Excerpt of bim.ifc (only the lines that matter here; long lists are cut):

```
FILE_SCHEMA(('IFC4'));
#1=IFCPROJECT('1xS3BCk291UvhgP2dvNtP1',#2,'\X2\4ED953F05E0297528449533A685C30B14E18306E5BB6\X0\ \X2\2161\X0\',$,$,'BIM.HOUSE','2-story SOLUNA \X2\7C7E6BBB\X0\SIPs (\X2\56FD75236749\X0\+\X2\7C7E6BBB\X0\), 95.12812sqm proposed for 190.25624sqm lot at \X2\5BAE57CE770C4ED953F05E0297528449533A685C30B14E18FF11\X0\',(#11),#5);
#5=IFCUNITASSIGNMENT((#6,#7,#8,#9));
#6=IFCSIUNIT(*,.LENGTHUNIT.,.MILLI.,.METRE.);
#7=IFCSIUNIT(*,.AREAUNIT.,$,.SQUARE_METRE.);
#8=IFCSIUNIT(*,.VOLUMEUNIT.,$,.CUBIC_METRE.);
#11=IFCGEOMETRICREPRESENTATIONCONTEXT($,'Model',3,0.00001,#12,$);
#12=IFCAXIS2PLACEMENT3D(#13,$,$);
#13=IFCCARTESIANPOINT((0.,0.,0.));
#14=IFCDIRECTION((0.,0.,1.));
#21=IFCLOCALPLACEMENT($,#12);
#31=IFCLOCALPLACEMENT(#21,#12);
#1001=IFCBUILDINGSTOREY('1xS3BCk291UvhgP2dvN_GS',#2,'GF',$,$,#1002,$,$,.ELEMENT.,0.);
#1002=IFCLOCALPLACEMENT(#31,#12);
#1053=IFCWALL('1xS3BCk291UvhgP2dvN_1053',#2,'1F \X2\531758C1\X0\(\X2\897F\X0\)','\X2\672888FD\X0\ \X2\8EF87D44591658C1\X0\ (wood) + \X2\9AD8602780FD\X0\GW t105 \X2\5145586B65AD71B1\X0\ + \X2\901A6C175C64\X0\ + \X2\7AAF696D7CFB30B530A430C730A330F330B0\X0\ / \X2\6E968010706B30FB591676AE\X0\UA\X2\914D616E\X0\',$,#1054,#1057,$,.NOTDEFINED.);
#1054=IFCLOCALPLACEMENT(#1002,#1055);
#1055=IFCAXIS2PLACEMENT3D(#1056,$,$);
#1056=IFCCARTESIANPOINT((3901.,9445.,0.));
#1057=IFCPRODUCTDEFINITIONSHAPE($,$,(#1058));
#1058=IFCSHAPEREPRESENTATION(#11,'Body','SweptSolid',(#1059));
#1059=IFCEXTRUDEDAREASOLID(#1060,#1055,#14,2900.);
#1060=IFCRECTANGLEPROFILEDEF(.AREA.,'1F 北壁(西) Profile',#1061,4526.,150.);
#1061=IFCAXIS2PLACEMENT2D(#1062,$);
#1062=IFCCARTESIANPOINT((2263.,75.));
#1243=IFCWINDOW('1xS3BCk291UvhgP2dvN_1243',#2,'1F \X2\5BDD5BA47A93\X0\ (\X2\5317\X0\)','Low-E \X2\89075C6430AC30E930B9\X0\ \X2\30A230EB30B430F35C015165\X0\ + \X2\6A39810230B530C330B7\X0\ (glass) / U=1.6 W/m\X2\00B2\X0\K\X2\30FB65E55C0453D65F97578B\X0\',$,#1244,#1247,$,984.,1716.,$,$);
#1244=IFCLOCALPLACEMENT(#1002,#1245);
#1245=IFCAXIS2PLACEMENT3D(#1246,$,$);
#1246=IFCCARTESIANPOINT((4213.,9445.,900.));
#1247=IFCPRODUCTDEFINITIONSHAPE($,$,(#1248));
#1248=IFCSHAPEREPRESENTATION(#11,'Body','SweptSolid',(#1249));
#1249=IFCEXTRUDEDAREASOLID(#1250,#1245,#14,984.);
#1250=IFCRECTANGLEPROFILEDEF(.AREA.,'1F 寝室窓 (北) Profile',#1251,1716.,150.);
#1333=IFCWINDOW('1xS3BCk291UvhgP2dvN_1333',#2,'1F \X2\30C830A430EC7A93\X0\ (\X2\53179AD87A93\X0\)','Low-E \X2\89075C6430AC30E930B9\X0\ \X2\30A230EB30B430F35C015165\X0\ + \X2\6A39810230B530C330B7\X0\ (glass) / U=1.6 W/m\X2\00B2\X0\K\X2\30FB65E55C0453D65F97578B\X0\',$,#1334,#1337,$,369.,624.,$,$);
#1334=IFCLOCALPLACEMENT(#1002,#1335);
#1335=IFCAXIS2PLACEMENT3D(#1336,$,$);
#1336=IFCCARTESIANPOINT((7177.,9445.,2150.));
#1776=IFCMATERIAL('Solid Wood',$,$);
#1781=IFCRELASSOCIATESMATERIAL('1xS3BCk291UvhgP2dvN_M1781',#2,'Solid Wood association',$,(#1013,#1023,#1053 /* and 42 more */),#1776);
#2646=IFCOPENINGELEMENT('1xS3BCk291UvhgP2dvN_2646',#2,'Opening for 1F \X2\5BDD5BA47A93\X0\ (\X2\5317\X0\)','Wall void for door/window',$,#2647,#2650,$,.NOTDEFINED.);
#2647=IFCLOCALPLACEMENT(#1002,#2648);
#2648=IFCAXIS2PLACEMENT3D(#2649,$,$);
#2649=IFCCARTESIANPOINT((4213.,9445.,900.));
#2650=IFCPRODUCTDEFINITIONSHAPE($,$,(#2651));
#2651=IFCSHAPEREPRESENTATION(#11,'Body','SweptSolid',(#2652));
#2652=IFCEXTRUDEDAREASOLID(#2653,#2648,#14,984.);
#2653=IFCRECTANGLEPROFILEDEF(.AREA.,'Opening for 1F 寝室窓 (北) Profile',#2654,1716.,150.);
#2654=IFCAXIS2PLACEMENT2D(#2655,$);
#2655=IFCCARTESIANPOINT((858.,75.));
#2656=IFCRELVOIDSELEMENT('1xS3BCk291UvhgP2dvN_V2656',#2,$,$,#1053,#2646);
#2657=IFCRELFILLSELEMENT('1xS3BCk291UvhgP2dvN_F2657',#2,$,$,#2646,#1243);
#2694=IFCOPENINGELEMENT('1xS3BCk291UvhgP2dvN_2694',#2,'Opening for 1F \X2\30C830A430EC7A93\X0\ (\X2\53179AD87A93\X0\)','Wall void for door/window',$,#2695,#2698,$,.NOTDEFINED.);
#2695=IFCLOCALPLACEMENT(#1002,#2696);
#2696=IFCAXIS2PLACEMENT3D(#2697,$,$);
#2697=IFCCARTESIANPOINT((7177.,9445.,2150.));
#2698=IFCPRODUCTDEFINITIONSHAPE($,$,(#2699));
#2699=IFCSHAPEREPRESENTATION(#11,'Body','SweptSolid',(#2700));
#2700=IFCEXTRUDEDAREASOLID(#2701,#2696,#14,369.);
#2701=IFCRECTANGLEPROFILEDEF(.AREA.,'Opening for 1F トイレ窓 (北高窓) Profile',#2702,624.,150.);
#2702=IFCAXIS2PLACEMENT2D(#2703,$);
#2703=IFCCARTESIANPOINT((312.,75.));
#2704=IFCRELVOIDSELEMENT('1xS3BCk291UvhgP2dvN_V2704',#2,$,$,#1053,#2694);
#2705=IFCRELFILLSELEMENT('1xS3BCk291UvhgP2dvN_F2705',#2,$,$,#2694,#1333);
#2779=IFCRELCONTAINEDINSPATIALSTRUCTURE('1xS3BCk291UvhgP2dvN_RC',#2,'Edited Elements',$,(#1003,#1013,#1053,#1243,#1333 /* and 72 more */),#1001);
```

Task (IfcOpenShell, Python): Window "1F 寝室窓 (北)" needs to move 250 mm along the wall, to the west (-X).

```python
import ifcopenshell
import ifcopenshell.api.geometry
import ifcopenshell.util.placement

model = ifcopenshell.open("bim.ifc")

window = model.by_guid("1xS3BCk291UvhgP2dvN_1243")
opening = window.FillsVoids[0].RelatingOpeningElement
wall = opening.VoidsElements[0].RelatingBuildingElement

wall_matrix = ifcopenshell.util.placement.get_local_placement(wall.ObjectPlacement)
shift = wall_matrix[:3, 0] * -250.0
before = ifcopenshell.util.placement.get_local_placement(window.ObjectPlacement)[:3, 3].copy()

# The window is not placed relative to its opening, so move both.
for product in (opening, window):
    matrix = ifcopenshell.util.placement.get_local_placement(product.ObjectPlacement)
    matrix[:3, 3] += shift
    ifcopenshell.api.geometry.edit_object_placement(model, product=product, matrix=matrix, is_si=False)

after = ifcopenshell.util.placement.get_local_placement(window.ObjectPlacement)[:3, 3]
print("window moved by", (after - before).round(3) + 0.0)

model.write("bim_v2.ifc")
```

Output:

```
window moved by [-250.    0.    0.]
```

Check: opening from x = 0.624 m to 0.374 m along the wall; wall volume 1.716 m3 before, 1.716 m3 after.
